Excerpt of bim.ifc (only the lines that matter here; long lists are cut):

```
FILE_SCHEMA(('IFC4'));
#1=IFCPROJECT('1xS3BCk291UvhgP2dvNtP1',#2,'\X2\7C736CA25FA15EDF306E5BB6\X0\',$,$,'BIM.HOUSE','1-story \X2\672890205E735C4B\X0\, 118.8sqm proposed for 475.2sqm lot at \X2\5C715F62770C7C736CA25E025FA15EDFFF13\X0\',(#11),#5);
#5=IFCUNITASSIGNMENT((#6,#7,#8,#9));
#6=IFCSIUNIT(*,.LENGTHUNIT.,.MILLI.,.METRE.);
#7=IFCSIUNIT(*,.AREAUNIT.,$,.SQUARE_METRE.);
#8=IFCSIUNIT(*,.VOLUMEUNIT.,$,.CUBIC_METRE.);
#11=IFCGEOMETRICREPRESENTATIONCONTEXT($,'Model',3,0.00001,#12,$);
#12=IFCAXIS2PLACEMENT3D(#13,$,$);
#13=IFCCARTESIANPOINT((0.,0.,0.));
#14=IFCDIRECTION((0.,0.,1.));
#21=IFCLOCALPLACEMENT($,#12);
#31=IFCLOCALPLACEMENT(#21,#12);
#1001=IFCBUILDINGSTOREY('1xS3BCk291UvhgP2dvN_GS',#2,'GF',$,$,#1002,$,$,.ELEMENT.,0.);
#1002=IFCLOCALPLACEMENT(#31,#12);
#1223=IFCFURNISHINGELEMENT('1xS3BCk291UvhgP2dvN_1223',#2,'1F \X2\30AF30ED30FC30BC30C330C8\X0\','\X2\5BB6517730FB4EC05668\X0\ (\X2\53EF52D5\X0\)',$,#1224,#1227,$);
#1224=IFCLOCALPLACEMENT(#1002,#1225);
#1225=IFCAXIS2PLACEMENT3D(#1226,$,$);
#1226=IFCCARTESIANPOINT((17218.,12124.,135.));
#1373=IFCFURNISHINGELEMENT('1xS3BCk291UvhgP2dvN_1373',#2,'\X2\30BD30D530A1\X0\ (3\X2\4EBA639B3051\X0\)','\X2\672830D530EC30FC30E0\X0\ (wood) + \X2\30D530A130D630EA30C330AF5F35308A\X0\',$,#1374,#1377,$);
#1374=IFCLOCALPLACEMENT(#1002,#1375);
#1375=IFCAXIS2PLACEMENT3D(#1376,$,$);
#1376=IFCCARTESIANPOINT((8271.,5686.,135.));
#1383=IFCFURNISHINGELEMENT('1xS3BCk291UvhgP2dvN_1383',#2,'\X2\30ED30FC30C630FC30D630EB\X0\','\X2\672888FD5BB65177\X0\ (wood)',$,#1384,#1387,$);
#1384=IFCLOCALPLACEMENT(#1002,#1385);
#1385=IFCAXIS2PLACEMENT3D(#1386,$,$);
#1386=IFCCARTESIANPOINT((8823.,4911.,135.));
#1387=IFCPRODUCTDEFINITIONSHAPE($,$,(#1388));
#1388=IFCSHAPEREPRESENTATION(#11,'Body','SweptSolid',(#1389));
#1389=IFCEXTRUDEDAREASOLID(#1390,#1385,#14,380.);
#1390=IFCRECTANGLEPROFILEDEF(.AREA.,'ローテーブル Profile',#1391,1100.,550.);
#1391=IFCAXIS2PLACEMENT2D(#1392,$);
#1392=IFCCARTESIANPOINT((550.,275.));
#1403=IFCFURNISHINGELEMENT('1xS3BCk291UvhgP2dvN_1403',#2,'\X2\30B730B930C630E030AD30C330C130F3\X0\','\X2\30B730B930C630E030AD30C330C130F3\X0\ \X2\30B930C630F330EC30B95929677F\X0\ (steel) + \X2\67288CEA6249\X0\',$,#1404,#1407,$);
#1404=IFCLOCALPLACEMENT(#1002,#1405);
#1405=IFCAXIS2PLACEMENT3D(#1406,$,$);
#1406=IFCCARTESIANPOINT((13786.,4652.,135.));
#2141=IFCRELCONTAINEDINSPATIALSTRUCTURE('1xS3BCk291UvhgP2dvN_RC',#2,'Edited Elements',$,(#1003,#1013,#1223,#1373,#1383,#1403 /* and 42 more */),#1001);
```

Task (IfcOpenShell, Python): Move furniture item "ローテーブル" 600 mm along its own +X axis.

```python
import ifcopenshell
import ifcopenshell.api.geometry
import ifcopenshell.util.placement
import ifcopenshell.util.unit

model = ifcopenshell.open("bim.ifc")
unit_scale = ifcopenshell.util.unit.calculate_unit_scale(model)

item = model.by_guid("1xS3BCk291UvhgP2dvN_1383")
matrix = ifcopenshell.util.placement.get_local_placement(item.ObjectPlacement)
matrix[:3, 3] += matrix[:3, 0] * 0.6 / unit_scale
ifcopenshell.api.geometry.edit_object_placement(model, product=item, matrix=matrix, is_si=False)

print(ifcopenshell.util.placement.get_local_placement(item.ObjectPlacement).round(3) + 0.0)

model.write("bim_edited.ifc")
```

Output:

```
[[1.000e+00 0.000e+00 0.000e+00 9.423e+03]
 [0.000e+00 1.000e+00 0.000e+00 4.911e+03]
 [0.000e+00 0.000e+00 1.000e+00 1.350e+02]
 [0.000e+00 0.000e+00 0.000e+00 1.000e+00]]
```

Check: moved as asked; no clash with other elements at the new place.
